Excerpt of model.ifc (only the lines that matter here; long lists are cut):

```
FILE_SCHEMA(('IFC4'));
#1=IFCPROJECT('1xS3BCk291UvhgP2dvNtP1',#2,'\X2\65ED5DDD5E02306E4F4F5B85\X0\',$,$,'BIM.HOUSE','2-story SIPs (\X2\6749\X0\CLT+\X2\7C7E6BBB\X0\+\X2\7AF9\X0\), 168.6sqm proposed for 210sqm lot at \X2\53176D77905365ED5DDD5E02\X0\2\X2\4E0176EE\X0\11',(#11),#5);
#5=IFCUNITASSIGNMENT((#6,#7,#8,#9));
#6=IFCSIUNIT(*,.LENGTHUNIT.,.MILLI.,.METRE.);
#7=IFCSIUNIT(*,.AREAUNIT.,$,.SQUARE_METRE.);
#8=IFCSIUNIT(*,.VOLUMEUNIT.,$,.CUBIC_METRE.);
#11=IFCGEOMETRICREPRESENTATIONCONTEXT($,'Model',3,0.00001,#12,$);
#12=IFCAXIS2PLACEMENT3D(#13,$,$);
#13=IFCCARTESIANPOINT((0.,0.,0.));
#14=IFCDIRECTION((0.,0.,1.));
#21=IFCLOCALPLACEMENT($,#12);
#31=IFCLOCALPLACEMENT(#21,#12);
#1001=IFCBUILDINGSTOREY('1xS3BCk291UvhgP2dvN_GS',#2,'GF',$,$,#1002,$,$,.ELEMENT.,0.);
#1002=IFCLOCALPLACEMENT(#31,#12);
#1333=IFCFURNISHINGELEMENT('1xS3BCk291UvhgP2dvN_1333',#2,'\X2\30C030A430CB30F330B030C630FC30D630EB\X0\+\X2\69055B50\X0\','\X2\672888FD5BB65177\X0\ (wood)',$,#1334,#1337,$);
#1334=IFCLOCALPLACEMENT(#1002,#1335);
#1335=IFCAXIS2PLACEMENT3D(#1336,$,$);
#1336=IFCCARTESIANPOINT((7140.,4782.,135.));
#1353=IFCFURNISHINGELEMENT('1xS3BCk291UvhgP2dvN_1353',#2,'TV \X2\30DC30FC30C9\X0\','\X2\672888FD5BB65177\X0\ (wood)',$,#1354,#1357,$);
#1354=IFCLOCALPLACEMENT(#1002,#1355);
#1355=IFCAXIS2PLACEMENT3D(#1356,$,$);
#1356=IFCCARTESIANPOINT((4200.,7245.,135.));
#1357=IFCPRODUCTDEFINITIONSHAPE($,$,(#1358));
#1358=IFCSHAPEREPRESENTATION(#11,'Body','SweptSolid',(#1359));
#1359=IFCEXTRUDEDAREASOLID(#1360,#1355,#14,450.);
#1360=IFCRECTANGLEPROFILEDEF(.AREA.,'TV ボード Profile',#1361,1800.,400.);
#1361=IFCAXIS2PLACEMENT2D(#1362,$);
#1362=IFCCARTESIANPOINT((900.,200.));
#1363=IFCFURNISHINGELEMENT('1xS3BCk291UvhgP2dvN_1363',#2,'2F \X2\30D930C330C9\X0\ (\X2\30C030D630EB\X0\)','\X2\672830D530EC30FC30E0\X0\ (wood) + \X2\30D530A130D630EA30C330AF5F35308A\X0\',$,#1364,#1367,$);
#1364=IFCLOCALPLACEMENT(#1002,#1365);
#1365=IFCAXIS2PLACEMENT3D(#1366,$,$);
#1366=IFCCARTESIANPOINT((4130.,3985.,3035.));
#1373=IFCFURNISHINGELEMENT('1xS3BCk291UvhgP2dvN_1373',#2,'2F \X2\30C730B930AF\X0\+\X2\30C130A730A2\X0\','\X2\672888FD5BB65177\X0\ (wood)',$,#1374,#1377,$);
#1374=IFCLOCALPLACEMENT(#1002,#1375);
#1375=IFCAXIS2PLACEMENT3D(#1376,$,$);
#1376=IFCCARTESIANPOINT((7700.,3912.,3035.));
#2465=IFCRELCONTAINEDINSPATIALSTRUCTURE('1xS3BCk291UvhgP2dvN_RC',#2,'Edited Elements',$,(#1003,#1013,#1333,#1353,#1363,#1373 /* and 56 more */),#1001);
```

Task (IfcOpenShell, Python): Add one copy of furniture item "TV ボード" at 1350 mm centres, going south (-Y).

```python
import numpy as np
import ifcopenshell
import ifcopenshell.api.geometry
import ifcopenshell.api.root
import ifcopenshell.util.element
import ifcopenshell.util.placement

model = ifcopenshell.open("model.ifc")


def reuse_history(source, copy):
    """copy_class also copies each property set's owner history, people and application; keep the originals."""
    for rel in copy.IsDefinedBy:
        if rel.is_a("IfcRelDefinesByProperties") and (history := rel.RelatingPropertyDefinition.OwnerHistory):
            rel.RelatingPropertyDefinition.OwnerHistory = source.OwnerHistory
            ifcopenshell.util.element.remove_deep2(model, history)


source = model.by_guid("1xS3BCk291UvhgP2dvN_1353")
base = ifcopenshell.util.placement.get_local_placement(source.ObjectPlacement)
step = np.array([0.0, -1.0, 0.0]) * 1350.0

for i in range(1, 2):
    copy = ifcopenshell.api.root.copy_class(model, product=source)
    copy.Representation = ifcopenshell.util.element.copy_deep(
        model, source.Representation, exclude=["IfcGeometricRepresentationContext", "IfcRepresentationMap"]
    )
    reuse_history(source, copy)
    matrix = base.copy()
    matrix[:3, 3] += i * step
    print("added at", matrix[:3, 3].round(3) + 0.0)
    ifcopenshell.api.geometry.edit_object_placement(model, product=copy, matrix=matrix, is_si=False)

model.write("model_rev.ifc")
```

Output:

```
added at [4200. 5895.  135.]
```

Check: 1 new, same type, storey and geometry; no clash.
